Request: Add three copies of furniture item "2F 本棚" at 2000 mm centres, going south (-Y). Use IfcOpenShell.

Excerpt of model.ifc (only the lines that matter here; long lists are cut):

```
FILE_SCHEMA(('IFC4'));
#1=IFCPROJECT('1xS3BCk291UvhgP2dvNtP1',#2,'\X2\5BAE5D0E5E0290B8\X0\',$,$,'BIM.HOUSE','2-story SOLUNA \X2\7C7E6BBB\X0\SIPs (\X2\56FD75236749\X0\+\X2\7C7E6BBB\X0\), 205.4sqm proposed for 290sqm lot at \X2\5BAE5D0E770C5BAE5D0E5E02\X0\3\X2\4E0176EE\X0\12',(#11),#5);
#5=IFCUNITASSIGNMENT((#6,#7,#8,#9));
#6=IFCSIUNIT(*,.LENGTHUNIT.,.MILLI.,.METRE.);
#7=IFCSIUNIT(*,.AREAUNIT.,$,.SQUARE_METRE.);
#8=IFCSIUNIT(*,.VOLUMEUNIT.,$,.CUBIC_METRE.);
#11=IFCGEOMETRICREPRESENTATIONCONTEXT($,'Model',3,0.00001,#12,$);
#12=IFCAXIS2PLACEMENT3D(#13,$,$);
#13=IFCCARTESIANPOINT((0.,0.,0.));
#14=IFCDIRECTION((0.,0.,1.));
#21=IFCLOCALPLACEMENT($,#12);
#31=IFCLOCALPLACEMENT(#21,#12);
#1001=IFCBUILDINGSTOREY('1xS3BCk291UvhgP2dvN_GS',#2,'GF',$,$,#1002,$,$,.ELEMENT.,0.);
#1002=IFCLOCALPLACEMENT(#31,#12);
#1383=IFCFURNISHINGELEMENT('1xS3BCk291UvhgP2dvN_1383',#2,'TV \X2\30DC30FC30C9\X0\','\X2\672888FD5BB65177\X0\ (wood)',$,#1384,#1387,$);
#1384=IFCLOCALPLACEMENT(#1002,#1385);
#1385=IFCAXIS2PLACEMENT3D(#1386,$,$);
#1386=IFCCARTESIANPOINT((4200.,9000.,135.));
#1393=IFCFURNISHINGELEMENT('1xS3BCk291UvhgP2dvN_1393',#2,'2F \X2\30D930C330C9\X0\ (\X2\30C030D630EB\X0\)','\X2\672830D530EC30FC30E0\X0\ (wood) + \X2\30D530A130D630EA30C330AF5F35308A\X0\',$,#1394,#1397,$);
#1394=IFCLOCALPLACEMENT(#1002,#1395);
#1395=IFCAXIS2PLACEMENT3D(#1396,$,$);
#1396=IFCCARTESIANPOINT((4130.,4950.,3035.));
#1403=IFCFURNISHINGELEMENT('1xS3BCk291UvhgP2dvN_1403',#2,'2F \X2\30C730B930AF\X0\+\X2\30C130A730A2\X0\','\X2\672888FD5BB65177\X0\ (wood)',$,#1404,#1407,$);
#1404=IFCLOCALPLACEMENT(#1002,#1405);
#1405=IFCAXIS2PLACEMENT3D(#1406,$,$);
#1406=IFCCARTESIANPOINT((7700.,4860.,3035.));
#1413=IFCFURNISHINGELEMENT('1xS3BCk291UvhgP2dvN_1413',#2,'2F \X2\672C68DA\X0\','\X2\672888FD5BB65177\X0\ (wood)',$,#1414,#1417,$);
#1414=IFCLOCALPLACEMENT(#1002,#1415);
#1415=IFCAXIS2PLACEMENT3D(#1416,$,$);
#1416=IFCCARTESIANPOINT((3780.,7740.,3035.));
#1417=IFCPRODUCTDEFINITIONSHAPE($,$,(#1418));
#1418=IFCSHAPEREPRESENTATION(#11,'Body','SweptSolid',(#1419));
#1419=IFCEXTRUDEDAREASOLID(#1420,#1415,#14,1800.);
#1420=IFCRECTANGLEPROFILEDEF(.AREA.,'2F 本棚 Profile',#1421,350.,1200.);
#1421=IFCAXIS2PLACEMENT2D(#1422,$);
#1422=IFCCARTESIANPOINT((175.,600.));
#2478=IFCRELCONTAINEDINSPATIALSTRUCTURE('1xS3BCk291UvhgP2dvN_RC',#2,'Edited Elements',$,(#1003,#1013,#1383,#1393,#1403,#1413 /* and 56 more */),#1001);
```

```python
import numpy as np
import ifcopenshell
import ifcopenshell.api.geometry
import ifcopenshell.api.root
import ifcopenshell.util.element
import ifcopenshell.util.placement
import ifcopenshell.util.unit

model = ifcopenshell.open("model.ifc")
unit_scale = ifcopenshell.util.unit.calculate_unit_scale(model)


def reuse_history(source, copy):
    """copy_class also copies each property set's owner history, people and application; keep the originals."""
    for rel in copy.IsDefinedBy:
        if rel.is_a("IfcRelDefinesByProperties") and (history := rel.RelatingPropertyDefinition.OwnerHistory):
            rel.RelatingPropertyDefinition.OwnerHistory = source.OwnerHistory
            ifcopenshell.util.element.remove_deep2(model, history)


source = model.by_guid("1xS3BCk291UvhgP2dvN_1413")
base = ifcopenshell.util.placement.get_local_placement(source.ObjectPlacement)
step = np.array([0.0, -1.0, 0.0]) * 2 / unit_scale

for i in range(1, 4):
    copy = ifcopenshell.api.root.copy_class(model, product=source)
    copy.Representation = ifcopenshell.util.element.copy_deep(
        model, source.Representation, exclude=["IfcGeometricRepresentationContext", "IfcRepresentationMap"]
    )
    reuse_history(source, copy)
    matrix = base.copy()
    matrix[:3, 3] += i * step
    print("added at", matrix[:3, 3].round(3) + 0.0)
    ifcopenshell.api.geometry.edit_object_placement(model, product=copy, matrix=matrix, is_si=False)

model.write("model_edited.ifc")
```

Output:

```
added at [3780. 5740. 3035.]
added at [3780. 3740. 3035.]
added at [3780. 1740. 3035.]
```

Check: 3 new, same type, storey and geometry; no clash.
